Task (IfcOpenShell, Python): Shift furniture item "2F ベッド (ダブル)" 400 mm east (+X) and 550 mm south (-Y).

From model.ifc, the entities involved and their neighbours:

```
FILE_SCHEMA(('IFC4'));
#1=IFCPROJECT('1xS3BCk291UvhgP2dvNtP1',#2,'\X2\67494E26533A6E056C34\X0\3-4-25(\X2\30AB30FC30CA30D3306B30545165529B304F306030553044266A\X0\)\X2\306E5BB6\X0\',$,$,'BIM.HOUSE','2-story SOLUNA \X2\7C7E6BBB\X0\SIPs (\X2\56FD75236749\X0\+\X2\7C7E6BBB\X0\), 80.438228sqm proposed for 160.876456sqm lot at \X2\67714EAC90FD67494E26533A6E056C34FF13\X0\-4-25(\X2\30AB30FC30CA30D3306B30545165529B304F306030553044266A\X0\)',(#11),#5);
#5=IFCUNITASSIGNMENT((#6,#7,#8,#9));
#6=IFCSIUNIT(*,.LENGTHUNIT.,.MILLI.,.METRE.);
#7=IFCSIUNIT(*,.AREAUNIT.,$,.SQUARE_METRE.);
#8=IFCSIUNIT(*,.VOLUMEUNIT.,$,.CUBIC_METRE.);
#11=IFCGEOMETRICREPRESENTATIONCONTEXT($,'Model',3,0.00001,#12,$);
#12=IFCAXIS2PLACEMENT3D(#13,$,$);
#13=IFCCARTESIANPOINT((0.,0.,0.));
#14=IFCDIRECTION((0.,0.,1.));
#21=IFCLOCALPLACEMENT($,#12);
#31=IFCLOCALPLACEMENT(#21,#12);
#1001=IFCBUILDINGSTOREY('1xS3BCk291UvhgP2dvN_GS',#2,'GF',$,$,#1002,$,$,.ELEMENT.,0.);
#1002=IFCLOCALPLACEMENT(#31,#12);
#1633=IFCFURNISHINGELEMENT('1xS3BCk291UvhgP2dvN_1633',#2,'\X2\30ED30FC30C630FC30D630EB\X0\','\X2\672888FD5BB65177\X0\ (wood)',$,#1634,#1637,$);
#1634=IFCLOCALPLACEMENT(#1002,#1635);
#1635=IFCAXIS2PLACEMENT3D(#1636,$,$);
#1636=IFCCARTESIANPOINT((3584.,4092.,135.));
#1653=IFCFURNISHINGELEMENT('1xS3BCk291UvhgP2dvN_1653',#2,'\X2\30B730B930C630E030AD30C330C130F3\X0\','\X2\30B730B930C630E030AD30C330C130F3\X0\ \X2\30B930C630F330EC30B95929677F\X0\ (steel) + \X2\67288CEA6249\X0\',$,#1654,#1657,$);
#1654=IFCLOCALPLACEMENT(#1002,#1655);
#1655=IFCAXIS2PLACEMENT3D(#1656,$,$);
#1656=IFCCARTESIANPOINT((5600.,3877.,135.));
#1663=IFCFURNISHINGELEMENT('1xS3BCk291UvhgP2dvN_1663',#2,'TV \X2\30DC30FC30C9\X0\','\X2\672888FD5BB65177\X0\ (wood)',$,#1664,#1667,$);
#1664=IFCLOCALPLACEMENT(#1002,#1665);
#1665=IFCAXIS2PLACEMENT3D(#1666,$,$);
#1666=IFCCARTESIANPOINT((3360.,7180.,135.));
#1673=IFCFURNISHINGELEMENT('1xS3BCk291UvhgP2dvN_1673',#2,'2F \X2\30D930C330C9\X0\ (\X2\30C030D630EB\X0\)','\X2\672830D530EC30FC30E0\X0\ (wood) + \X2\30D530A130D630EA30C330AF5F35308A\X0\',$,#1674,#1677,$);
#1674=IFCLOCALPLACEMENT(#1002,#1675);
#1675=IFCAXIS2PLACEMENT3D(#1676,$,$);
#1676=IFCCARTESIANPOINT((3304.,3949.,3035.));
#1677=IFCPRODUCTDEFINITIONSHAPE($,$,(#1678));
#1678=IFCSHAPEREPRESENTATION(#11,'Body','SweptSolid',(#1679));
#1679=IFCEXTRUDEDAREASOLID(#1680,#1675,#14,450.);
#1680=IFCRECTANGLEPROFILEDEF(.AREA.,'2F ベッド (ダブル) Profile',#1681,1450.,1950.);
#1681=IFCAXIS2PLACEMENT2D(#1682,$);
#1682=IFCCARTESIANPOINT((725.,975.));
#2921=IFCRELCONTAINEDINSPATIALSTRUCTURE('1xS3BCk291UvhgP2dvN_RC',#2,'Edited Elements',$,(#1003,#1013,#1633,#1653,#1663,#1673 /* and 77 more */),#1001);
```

```python
import ifcopenshell
import ifcopenshell.api.geometry
import ifcopenshell.util.placement

model = ifcopenshell.open("model.ifc")

item = model.by_guid("1xS3BCk291UvhgP2dvN_1673")
matrix = ifcopenshell.util.placement.get_local_placement(item.ObjectPlacement)
matrix[0, 3] += 400.0
matrix[1, 3] -= 550.0
ifcopenshell.api.geometry.edit_object_placement(model, product=item, matrix=matrix, is_si=False)

print(ifcopenshell.util.placement.get_local_placement(item.ObjectPlacement).round(3) + 0.0)

model.write("model_rev.ifc")
```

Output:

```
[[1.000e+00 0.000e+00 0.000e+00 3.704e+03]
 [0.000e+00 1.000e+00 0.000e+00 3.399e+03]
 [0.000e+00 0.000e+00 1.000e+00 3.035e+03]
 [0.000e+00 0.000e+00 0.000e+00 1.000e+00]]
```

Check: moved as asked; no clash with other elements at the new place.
